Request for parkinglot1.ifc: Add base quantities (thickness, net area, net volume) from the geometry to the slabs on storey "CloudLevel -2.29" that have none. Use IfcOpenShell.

First a look at what the model holds.

```python
import ifcopenshell
import ifcopenshell.util.element
import ifcopenshell.util.unit

model = ifcopenshell.open("parkinglot1.ifc")
print(model.schema)
for unit_type in ("LENGTHUNIT", "AREAUNIT", "VOLUMEUNIT"):
    print(unit_type, ifcopenshell.util.unit.calculate_unit_scale(model, unit_type))
storey = next(s for s in model.by_type("IfcBuildingStorey") if s.Name == "CloudLevel -2.29")
slabs = [e for e in ifcopenshell.util.element.get_decomposition(storey) if e.is_a("IfcSlab")]
for e in sorted(slabs, key=lambda e: e.id()):
    print(e.id(), e.is_a(), e.Name, list(ifcopenshell.util.element.get_psets(e, qtos_only=True)), sep=" | ")
```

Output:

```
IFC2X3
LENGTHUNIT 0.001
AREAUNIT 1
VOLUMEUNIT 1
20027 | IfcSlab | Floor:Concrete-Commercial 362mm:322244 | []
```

```python
import ifcopenshell
import ifcopenshell.api.pset
import ifcopenshell.geom
import ifcopenshell.util.element
import ifcopenshell.util.shape
import ifcopenshell.util.unit

model = ifcopenshell.open("parkinglot1.ifc")
unit_scale = ifcopenshell.util.unit.calculate_unit_scale(model)
area_scale = ifcopenshell.util.unit.calculate_unit_scale(model, "AREAUNIT")
volume_scale = ifcopenshell.util.unit.calculate_unit_scale(model, "VOLUMEUNIT")
settings = ifcopenshell.geom.settings()

storey = next(s for s in model.by_type("IfcBuildingStorey") if s.Name == "CloudLevel -2.29")
slabs = [e for e in ifcopenshell.util.element.get_decomposition(storey) if e.is_a("IfcSlab")]

for e in sorted(slabs, key=lambda e: e.id()):
    if ifcopenshell.util.element.get_psets(e, qtos_only=True, should_inherit=False):
        continue
    # Geometry comes back in metres, in the element's own axes.
    shape = ifcopenshell.geom.create_shape(settings, e)
    values = {
        "Width": ifcopenshell.util.shape.get_z(shape.geometry) / unit_scale,
        "NetArea": ifcopenshell.util.shape.get_footprint_area(shape.geometry) / area_scale,
        "NetVolume": ifcopenshell.util.shape.get_volume(shape.geometry) / volume_scale,
    }
    qto = ifcopenshell.api.pset.add_qto(model, product=e, name="BaseQuantities")
    ifcopenshell.api.pset.edit_qto(model, qto=qto, properties=values)
    print(e.id(), {k: round(v, 3) for k, v in values.items()})

model.write("parkinglot1_updated.ifc")
```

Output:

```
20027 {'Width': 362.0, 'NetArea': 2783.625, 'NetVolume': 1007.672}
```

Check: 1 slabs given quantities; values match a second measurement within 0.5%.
